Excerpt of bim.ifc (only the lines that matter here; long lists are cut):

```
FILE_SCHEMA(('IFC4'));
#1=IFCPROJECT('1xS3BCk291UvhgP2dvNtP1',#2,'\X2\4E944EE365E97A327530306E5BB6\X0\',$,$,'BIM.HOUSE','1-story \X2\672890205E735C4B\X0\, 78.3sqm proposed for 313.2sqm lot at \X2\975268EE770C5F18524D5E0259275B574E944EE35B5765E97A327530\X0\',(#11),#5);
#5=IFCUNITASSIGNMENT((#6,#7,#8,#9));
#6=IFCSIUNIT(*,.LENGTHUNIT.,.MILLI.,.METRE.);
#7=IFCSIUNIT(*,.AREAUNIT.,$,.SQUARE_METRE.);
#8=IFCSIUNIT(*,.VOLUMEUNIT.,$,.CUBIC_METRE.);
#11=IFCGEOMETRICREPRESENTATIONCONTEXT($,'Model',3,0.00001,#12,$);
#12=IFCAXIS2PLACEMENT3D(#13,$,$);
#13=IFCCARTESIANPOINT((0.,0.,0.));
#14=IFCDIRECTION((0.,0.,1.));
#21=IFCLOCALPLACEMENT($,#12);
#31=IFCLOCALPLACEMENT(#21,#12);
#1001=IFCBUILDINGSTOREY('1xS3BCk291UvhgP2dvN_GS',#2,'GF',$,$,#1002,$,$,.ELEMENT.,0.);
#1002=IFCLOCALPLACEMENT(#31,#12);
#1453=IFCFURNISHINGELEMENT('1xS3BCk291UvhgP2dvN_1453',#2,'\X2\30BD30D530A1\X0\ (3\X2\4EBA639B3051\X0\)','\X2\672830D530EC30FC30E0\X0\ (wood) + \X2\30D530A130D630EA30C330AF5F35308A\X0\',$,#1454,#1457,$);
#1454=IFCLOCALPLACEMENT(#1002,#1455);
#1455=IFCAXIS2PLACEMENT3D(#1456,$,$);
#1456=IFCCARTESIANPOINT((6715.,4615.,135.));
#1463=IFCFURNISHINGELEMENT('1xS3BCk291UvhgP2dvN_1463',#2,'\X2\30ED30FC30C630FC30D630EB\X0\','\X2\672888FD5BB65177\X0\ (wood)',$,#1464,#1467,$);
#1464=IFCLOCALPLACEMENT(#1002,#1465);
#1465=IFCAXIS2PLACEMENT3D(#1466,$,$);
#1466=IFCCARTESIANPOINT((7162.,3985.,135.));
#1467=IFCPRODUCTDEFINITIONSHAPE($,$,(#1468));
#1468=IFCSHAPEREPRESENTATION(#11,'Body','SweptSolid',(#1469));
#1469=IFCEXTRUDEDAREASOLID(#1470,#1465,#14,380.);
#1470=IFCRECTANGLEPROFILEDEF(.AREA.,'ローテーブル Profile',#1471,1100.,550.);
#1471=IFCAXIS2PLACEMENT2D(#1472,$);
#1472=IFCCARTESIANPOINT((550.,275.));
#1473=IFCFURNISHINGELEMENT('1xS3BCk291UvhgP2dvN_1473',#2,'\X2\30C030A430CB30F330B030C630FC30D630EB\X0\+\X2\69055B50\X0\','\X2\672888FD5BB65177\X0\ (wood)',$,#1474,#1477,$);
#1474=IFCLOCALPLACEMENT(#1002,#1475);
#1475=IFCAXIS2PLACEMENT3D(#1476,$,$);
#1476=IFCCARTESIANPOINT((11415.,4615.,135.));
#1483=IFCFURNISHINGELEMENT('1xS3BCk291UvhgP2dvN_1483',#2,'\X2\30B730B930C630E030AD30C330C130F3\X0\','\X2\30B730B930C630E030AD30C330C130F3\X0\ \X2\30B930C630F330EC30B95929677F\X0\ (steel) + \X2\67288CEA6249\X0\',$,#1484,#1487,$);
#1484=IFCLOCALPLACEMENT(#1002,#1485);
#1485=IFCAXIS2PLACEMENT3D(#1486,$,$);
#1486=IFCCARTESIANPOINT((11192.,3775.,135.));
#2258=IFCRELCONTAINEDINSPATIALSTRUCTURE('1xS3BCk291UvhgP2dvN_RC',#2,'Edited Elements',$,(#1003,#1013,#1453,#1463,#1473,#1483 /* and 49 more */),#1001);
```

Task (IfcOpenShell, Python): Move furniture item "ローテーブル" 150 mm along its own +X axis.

```python
import ifcopenshell
import ifcopenshell.api.geometry
import ifcopenshell.util.placement
import ifcopenshell.util.unit

model = ifcopenshell.open("bim.ifc")
unit_scale = ifcopenshell.util.unit.calculate_unit_scale(model)

item = model.by_id(1463)
matrix = ifcopenshell.util.placement.get_local_placement(item.ObjectPlacement)
matrix[:3, 3] += matrix[:3, 0] * 0.15 / unit_scale
ifcopenshell.api.geometry.edit_object_placement(model, product=item, matrix=matrix, is_si=False)

print(ifcopenshell.util.placement.get_local_placement(item.ObjectPlacement).round(3) + 0.0)

model.write("bim_v2.ifc")
```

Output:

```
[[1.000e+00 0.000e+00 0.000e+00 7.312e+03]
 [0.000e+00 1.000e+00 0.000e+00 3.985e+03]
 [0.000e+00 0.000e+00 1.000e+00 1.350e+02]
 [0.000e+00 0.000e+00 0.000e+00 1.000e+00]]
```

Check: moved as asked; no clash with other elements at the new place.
